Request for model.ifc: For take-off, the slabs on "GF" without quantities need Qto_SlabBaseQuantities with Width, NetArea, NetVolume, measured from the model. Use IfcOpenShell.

First a look at what the model holds.

```python
import ifcopenshell
import ifcopenshell.util.element
import ifcopenshell.util.unit

model = ifcopenshell.open("model.ifc")
print(model.schema)
for unit_type in ("LENGTHUNIT", "AREAUNIT", "VOLUMEUNIT"):
    print(unit_type, ifcopenshell.util.unit.calculate_unit_scale(model, unit_type))
storey = next(s for s in model.by_type("IfcBuildingStorey") if s.Name == "GF")
slabs = [e for e in ifcopenshell.util.element.get_decomposition(storey) if e.is_a("IfcSlab")]
for e in sorted(slabs, key=lambda e: e.id()):
    print(e.id(), e.is_a(), e.Name, list(ifcopenshell.util.element.get_psets(e, qtos_only=True)), sep=" | ")
```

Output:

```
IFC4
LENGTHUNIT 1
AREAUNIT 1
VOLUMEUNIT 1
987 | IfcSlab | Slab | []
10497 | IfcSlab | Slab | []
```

```python
import ifcopenshell
import ifcopenshell.api.pset
import ifcopenshell.geom
import ifcopenshell.util.element
import ifcopenshell.util.shape
import ifcopenshell.util.unit

model = ifcopenshell.open("model.ifc")
unit_scale = ifcopenshell.util.unit.calculate_unit_scale(model)
area_scale = ifcopenshell.util.unit.calculate_unit_scale(model, "AREAUNIT")
volume_scale = ifcopenshell.util.unit.calculate_unit_scale(model, "VOLUMEUNIT")
settings = ifcopenshell.geom.settings()

storey = next(s for s in model.by_type("IfcBuildingStorey") if s.Name == "GF")
slabs = [e for e in ifcopenshell.util.element.get_decomposition(storey) if e.is_a("IfcSlab")]

for e in sorted(slabs, key=lambda e: e.id()):
    if ifcopenshell.util.element.get_psets(e, qtos_only=True, should_inherit=False):
        continue
    # Geometry comes back in metres, in the element's own axes.
    shape = ifcopenshell.geom.create_shape(settings, e)
    values = {
        "Width": ifcopenshell.util.shape.get_z(shape.geometry) / unit_scale,
        "NetArea": ifcopenshell.util.shape.get_footprint_area(shape.geometry) / area_scale,
        "NetVolume": ifcopenshell.util.shape.get_volume(shape.geometry) / volume_scale,
    }
    qto = ifcopenshell.api.pset.add_qto(model, product=e, name="Qto_SlabBaseQuantities")
    ifcopenshell.api.pset.edit_qto(model, qto=qto, properties=values)
    print(e.id(), {k: round(v, 3) for k, v in values.items()})

model.write("model-out.ifc")
```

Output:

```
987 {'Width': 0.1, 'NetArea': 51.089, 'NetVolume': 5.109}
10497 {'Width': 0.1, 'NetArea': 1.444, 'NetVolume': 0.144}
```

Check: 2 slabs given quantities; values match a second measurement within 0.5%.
